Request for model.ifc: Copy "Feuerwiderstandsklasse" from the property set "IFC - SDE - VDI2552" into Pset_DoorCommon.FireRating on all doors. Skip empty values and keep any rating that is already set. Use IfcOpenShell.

First a look at what the model holds.

```python
import ifcopenshell
import ifcopenshell.util.element

model = ifcopenshell.open("model.ifc")
print(model.schema)
doors = model.by_type("IfcDoor")
print(len(doors), "doors")
for e in doors[:8]:
    source = ifcopenshell.util.element.get_pset(e, "IFC - SDE - VDI2552", "Feuerwiderstandsklasse")
    target = ifcopenshell.util.element.get_pset(e, "Pset_DoorCommon", "FireRating")
    print(e.id(), repr(source), repr(target), sep=" | ")
```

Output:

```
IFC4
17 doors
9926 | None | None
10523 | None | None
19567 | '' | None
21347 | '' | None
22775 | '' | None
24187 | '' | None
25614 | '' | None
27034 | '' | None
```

```python
import ifcopenshell
import ifcopenshell.api.pset
import ifcopenshell.util.element

model = ifcopenshell.open("model.ifc")

count = 0
for e in model.by_type("IfcDoor"):
    value = ifcopenshell.util.element.get_pset(e, "IFC - SDE - VDI2552", "Feuerwiderstandsklasse")
    current = ifcopenshell.util.element.get_pset(e, "Pset_DoorCommon", "FireRating")
    if not value or not value.strip() or current:
        continue
    # add_pset returns the element's existing set when there is one.
    pset = ifcopenshell.api.pset.add_pset(model, product=e, name="Pset_DoorCommon")
    ifcopenshell.api.pset.edit_pset(model, pset=pset, properties={"FireRating": value})
    count += 1

print(count, "doors updated")

model.write("model_updated.ifc")
```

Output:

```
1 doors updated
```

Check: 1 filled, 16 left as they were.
